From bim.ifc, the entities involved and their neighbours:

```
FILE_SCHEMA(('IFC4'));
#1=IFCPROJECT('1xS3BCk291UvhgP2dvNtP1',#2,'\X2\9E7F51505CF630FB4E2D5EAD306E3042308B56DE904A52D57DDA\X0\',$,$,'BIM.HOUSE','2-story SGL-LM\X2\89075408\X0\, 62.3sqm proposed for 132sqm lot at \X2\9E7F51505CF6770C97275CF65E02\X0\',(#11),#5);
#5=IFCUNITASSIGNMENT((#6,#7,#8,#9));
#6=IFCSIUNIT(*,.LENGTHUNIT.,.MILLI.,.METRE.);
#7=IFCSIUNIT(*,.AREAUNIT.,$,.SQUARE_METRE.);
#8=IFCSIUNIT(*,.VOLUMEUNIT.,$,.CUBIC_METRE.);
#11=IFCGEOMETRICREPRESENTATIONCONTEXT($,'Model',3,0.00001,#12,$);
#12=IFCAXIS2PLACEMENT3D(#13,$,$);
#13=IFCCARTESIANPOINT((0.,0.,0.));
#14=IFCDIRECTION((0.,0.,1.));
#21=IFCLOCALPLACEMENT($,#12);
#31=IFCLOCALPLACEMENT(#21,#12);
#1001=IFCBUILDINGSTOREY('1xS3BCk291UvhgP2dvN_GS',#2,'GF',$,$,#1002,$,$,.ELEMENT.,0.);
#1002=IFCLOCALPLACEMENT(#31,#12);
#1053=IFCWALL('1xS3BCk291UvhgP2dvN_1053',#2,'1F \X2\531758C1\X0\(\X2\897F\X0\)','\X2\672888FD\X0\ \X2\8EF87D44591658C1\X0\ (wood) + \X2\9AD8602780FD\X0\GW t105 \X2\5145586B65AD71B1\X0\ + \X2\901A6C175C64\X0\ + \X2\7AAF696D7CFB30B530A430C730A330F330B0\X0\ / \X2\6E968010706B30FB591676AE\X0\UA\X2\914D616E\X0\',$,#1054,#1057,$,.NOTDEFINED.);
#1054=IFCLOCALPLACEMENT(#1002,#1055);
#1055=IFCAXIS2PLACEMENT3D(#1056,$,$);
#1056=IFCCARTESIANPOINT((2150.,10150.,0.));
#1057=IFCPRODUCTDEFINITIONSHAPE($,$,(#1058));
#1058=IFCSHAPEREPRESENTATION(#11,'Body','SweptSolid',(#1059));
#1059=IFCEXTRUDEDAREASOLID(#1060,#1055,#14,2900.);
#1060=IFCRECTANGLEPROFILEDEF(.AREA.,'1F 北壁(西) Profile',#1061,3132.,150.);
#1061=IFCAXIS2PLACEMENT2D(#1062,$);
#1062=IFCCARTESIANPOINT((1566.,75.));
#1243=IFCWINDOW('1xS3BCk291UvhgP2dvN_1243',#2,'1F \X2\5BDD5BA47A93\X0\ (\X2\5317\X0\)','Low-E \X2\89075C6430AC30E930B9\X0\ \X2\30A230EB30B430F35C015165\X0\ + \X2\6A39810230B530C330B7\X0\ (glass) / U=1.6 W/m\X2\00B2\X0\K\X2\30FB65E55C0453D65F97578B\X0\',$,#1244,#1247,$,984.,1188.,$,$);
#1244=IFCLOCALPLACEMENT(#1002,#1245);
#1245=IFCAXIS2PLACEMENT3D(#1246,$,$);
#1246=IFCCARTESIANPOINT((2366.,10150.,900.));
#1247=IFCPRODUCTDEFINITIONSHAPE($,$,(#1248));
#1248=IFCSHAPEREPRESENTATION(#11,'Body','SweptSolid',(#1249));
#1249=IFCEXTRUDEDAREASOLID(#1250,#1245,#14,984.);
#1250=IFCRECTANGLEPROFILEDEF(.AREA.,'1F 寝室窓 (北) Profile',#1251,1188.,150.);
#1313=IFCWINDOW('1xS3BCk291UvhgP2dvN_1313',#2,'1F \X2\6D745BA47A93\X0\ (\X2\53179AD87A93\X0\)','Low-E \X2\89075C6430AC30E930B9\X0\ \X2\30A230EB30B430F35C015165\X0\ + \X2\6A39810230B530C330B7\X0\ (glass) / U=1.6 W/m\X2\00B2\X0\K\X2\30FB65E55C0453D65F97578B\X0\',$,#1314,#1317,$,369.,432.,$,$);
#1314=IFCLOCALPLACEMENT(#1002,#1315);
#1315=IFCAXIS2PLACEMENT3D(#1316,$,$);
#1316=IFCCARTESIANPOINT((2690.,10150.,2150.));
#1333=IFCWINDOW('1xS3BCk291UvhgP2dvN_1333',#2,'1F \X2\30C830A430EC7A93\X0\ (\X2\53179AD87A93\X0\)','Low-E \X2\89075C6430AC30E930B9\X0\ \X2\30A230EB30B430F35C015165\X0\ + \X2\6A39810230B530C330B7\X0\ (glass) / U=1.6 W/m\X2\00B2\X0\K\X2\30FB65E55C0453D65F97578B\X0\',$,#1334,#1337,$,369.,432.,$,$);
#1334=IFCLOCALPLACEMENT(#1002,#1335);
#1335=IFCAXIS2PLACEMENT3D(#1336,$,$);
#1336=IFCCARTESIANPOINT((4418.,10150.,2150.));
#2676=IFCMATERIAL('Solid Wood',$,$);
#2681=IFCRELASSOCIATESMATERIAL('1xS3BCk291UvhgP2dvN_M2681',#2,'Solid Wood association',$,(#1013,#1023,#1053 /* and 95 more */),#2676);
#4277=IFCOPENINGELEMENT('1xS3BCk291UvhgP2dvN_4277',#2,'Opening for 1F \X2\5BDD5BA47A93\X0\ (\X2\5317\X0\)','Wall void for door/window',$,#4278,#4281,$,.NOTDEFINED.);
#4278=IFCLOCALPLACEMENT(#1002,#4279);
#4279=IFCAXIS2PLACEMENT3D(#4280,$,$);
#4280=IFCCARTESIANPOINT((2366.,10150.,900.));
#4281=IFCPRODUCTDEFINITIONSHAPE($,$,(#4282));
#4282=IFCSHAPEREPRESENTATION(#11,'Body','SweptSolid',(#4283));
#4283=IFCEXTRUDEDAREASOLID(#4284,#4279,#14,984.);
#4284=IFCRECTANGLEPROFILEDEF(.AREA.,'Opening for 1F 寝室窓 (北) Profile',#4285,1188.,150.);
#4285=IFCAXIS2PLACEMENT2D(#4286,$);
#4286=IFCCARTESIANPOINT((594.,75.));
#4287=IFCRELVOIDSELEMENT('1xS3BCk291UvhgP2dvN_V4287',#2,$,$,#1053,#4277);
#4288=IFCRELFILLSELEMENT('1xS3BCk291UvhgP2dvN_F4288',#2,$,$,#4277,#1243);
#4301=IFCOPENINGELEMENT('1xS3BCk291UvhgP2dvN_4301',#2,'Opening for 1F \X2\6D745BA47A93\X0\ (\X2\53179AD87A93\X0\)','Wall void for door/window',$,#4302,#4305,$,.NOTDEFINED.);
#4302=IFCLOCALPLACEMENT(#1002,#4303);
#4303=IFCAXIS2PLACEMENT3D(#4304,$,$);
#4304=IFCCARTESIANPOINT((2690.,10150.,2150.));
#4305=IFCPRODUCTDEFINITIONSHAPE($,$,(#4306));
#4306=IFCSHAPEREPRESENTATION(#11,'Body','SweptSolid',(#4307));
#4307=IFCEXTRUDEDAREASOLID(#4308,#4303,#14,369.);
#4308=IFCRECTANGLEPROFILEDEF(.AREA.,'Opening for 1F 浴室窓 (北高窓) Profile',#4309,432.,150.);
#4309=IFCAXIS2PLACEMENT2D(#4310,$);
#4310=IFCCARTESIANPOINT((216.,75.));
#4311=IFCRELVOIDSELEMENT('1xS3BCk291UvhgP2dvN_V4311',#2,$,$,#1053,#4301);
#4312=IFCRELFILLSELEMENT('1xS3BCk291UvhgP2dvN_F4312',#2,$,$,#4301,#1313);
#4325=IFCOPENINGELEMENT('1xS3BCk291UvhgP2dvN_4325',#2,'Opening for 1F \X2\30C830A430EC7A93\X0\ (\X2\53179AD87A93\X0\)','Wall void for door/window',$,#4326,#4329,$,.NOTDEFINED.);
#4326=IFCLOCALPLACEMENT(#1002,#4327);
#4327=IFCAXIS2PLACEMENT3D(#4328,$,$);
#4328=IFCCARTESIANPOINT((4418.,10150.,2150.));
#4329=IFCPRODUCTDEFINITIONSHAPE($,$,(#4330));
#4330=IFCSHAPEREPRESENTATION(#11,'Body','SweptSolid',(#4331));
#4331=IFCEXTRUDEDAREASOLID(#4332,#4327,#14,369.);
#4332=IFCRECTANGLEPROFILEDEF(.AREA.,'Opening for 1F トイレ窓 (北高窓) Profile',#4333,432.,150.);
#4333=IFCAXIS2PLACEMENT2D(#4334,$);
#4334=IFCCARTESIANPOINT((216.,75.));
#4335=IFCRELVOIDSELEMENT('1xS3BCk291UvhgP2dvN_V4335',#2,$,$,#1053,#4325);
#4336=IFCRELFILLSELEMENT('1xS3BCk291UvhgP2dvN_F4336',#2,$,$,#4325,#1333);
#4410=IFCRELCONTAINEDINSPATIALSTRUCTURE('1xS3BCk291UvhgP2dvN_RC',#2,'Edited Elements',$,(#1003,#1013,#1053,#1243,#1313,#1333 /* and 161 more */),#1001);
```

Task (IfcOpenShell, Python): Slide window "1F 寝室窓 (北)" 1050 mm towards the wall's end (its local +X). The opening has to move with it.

```python
import ifcopenshell
import ifcopenshell.api.geometry
import ifcopenshell.util.placement

model = ifcopenshell.open("bim.ifc")

window = model.by_guid("1xS3BCk291UvhgP2dvN_1243")
opening = window.FillsVoids[0].RelatingOpeningElement
wall = opening.VoidsElements[0].RelatingBuildingElement

wall_matrix = ifcopenshell.util.placement.get_local_placement(wall.ObjectPlacement)
shift = wall_matrix[:3, 0] * 1050.0
before = ifcopenshell.util.placement.get_local_placement(window.ObjectPlacement)[:3, 3].copy()

# The window is not placed relative to its opening, so move both.
for product in (opening, window):
    matrix = ifcopenshell.util.placement.get_local_placement(product.ObjectPlacement)
    matrix[:3, 3] += shift
    ifcopenshell.api.geometry.edit_object_placement(model, product=product, matrix=matrix, is_si=False)

after = ifcopenshell.util.placement.get_local_placement(window.ObjectPlacement)[:3, 3]
print("window moved by", (after - before).round(3) + 0.0)

model.write("bim_v2.ifc")
```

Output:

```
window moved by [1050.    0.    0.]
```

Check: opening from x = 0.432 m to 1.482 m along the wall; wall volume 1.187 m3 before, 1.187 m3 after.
